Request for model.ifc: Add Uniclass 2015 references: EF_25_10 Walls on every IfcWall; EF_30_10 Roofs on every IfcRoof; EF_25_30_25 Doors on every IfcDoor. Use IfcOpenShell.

First a look at what the model holds.

```python
import ifcopenshell

model = ifcopenshell.open("model.ifc")
print(model.schema)
print("classifications:", [c.Name for c in model.by_type("IfcClassification")])
for ifc_class in ("IfcDoor", "IfcRoof", "IfcStair", "IfcWall", "IfcWindow"):
    print(ifc_class, len(model.by_type(ifc_class)))
```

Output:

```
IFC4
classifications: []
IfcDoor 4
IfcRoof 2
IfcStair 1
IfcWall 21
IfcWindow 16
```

```python
import ifcopenshell
import ifcopenshell.api.classification

model = ifcopenshell.open("model.ifc")

system = ifcopenshell.api.classification.add_classification(model, classification="Uniclass 2015")

codes = {
    "IfcWall": ("EF_25_10", "Walls"),
    "IfcRoof": ("EF_30_10", "Roofs"),
    "IfcDoor": ("EF_25_30_25", "Doors"),
}
for ifc_class, (code, name) in codes.items():
    products = model.by_type(ifc_class)
    ifcopenshell.api.classification.add_reference(
        model, products=products, classification=system, identification=code, name=name
    )
    print(code, len(products))

model.write("model_updated.ifc")
```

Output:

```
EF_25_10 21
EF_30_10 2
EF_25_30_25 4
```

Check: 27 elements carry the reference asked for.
